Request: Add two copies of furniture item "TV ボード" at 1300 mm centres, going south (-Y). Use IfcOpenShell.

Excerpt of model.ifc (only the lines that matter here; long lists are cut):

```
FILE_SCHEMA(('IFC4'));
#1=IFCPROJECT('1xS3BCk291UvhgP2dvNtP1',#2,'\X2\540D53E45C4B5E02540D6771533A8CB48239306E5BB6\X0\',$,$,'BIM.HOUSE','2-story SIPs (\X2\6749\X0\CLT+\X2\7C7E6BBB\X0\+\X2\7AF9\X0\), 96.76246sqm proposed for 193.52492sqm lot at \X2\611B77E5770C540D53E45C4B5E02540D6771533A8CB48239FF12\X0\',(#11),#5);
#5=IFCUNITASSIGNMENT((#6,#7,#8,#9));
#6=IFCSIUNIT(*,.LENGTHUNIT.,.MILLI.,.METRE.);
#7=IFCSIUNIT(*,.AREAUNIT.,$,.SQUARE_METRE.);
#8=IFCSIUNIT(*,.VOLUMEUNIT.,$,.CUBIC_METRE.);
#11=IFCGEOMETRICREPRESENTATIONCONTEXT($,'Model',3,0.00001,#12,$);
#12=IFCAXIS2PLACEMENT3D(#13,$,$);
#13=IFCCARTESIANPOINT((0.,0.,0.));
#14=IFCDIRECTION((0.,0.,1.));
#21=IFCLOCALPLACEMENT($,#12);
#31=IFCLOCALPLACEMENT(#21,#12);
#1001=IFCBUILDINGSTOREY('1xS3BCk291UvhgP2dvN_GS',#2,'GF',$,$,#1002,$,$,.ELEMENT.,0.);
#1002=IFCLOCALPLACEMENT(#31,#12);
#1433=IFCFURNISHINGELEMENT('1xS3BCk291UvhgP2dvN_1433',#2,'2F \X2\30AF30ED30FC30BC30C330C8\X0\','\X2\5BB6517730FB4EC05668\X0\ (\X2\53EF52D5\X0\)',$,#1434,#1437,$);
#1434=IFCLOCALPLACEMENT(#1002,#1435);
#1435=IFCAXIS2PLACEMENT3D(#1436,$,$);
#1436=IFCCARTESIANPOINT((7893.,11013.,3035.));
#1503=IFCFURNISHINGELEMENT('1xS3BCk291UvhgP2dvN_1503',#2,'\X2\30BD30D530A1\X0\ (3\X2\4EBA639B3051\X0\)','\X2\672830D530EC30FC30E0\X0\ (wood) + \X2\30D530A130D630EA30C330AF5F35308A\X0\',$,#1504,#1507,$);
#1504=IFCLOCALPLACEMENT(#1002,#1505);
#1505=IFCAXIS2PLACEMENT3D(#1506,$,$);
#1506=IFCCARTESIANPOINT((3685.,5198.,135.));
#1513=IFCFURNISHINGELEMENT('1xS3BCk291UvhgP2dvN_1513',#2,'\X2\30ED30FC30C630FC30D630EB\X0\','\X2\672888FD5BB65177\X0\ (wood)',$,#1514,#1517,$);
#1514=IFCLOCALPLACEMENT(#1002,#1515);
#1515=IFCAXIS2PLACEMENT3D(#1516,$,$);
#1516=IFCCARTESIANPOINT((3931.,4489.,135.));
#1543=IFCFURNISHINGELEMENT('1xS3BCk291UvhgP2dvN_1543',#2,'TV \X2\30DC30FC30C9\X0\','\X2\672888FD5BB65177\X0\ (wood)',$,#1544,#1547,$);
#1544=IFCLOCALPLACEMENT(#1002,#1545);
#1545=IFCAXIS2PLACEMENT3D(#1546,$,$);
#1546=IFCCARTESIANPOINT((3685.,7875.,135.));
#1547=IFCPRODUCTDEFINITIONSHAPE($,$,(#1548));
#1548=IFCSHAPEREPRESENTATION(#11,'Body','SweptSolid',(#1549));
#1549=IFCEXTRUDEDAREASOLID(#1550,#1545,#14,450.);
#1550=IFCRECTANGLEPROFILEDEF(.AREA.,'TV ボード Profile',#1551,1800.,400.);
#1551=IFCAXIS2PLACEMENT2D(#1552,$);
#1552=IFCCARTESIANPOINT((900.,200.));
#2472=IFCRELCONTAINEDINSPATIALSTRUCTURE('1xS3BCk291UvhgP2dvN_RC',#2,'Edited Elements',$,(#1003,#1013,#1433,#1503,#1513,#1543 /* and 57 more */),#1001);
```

```python
import numpy as np
import ifcopenshell
import ifcopenshell.api.geometry
import ifcopenshell.api.root
import ifcopenshell.util.element
import ifcopenshell.util.placement

model = ifcopenshell.open("model.ifc")


def reuse_history(source, copy):
    """copy_class also copies each property set's owner history, people and application; keep the originals."""
    for rel in copy.IsDefinedBy:
        if rel.is_a("IfcRelDefinesByProperties") and (history := rel.RelatingPropertyDefinition.OwnerHistory):
            rel.RelatingPropertyDefinition.OwnerHistory = source.OwnerHistory
            ifcopenshell.util.element.remove_deep2(model, history)


source = model.by_guid("1xS3BCk291UvhgP2dvN_1543")
base = ifcopenshell.util.placement.get_local_placement(source.ObjectPlacement)
step = np.array([0.0, -1.0, 0.0]) * 1300.0

for i in range(1, 3):
    copy = ifcopenshell.api.root.copy_class(model, product=source)
    copy.Representation = ifcopenshell.util.element.copy_deep(
        model, source.Representation, exclude=["IfcGeometricRepresentationContext", "IfcRepresentationMap"]
    )
    reuse_history(source, copy)
    matrix = base.copy()
    matrix[:3, 3] += i * step
    print("added at", matrix[:3, 3].round(3) + 0.0)
    ifcopenshell.api.geometry.edit_object_placement(model, product=copy, matrix=matrix, is_si=False)

model.write("model_rev.ifc")
```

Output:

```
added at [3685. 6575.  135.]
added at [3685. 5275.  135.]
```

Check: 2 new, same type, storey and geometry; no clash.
